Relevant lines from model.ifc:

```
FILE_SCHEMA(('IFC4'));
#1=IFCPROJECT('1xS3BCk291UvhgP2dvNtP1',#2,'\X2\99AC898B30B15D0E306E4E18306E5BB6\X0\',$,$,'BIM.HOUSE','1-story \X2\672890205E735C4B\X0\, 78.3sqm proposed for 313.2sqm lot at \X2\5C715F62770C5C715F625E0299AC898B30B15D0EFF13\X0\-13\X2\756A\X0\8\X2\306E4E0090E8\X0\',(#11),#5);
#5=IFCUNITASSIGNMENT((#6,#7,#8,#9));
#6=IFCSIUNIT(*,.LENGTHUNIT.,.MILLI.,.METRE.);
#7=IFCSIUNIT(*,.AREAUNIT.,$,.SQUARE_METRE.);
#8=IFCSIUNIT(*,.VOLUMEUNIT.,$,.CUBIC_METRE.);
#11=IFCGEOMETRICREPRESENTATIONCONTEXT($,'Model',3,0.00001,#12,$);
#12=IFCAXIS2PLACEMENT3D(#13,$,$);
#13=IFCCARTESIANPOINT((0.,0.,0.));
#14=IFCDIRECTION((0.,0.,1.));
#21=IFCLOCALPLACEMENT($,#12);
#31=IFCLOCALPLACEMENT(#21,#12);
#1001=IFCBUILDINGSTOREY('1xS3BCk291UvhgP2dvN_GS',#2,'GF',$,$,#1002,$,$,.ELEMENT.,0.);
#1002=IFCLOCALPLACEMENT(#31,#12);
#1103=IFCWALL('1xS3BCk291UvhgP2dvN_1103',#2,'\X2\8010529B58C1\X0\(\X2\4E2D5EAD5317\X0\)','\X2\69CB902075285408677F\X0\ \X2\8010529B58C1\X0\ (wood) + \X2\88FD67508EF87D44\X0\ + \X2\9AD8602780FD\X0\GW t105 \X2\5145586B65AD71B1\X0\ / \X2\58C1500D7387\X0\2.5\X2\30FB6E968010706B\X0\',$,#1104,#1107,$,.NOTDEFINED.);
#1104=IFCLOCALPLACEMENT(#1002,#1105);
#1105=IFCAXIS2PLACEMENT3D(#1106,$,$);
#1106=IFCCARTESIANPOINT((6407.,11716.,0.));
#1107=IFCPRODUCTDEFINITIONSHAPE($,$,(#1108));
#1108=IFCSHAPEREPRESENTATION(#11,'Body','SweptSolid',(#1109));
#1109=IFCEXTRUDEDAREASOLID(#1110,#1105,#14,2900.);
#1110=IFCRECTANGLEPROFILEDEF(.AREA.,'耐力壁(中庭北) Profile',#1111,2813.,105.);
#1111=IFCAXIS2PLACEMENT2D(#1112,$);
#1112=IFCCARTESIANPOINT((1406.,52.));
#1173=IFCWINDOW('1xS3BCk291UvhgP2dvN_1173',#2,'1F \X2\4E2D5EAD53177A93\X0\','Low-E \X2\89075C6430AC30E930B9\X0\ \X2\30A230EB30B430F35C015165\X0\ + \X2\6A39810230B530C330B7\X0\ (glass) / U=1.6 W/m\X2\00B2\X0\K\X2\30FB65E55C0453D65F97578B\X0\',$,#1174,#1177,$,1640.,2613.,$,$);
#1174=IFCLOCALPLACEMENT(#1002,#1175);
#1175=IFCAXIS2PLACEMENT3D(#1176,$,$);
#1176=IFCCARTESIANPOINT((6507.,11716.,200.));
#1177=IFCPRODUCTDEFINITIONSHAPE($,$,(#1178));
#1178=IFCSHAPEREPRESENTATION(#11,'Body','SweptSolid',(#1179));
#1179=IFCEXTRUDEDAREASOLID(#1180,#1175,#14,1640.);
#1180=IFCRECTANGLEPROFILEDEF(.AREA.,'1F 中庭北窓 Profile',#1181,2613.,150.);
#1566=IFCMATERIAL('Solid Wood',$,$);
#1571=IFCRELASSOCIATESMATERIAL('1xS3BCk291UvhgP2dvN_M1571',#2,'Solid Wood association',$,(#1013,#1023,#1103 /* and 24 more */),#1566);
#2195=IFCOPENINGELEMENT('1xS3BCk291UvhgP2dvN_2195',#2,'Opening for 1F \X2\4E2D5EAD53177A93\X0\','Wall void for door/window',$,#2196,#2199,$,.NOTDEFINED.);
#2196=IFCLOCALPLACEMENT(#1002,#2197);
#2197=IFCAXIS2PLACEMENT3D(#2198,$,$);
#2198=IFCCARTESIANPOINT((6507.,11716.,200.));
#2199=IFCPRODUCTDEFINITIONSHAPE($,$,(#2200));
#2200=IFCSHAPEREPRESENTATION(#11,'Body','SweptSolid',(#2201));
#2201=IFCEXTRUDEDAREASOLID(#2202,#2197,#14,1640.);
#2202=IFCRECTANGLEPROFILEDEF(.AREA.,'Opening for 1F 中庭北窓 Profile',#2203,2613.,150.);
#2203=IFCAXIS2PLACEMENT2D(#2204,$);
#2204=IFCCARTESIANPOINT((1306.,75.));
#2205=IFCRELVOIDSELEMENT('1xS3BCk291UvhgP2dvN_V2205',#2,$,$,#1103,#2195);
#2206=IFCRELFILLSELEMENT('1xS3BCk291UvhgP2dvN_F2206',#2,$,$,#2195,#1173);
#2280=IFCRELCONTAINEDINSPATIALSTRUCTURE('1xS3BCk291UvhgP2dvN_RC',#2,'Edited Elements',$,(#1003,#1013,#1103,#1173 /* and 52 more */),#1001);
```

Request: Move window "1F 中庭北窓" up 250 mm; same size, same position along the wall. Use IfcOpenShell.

```python
import numpy as np
import ifcopenshell
import ifcopenshell.api.geometry
import ifcopenshell.util.placement
import ifcopenshell.util.unit

model = ifcopenshell.open("model.ifc")
unit_scale = ifcopenshell.util.unit.calculate_unit_scale(model)

window = model.by_guid("1xS3BCk291UvhgP2dvN_1173")
opening = window.FillsVoids[0].RelatingOpeningElement
dz = 0.25 / unit_scale

shift = np.array([0.0, 0.0, dz])
# The window is not placed relative to its opening, so move both.
for product in (opening, window):
    matrix = ifcopenshell.util.placement.get_local_placement(product.ObjectPlacement)
    matrix[:3, 3] += shift
    ifcopenshell.api.geometry.edit_object_placement(model, product=product, matrix=matrix, is_si=False)

print(f"moved by {dz * unit_scale:+.3f} m")

model.write("model_rev.ifc")
```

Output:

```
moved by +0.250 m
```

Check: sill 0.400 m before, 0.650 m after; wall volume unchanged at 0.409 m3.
